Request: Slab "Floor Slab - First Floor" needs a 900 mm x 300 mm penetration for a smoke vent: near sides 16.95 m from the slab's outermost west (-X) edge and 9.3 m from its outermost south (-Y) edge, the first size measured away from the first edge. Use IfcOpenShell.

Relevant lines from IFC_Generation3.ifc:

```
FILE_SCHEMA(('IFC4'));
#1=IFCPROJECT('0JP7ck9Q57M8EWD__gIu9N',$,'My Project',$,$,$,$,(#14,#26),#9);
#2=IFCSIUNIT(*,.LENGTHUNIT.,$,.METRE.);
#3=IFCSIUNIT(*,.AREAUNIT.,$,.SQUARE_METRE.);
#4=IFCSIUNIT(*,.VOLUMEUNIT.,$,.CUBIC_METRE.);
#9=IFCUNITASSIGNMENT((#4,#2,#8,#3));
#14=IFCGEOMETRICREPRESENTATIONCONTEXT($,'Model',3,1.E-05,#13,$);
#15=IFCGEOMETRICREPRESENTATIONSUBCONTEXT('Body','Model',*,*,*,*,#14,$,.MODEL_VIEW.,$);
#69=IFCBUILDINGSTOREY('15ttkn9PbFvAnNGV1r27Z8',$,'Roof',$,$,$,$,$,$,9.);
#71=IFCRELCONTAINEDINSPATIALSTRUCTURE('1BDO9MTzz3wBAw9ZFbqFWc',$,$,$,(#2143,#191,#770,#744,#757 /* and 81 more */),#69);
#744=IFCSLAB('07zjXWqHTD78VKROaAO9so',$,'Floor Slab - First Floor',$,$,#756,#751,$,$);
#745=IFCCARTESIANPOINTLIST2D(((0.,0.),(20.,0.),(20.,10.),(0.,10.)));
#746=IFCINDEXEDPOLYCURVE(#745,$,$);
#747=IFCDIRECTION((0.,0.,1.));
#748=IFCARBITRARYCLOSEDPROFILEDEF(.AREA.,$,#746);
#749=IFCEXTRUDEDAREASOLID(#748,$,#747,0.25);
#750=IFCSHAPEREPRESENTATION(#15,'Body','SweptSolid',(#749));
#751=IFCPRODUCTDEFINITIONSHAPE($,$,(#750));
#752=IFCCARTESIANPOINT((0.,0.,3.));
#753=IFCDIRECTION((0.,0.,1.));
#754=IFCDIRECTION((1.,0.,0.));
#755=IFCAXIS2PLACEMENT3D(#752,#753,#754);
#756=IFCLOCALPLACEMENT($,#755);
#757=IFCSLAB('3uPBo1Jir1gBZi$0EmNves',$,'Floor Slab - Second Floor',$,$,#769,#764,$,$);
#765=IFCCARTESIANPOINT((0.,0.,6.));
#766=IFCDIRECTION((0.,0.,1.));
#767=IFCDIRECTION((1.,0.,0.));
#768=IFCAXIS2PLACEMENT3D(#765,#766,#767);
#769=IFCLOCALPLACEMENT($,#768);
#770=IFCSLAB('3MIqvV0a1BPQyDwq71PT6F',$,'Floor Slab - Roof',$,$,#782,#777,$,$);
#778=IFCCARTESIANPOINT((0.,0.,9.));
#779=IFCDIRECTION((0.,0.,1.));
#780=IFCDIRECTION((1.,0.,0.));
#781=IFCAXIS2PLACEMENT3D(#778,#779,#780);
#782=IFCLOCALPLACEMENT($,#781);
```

```python
import numpy as np
import ifcopenshell
import ifcopenshell.api.feature
import ifcopenshell.api.geometry
import ifcopenshell.api.root
import ifcopenshell.geom
import ifcopenshell.util.placement
import ifcopenshell.util.representation
import ifcopenshell.util.shape
import ifcopenshell.util.unit

model = ifcopenshell.open("IFC_Generation3.ifc")
unit_scale = ifcopenshell.util.unit.calculate_unit_scale(model)
settings = ifcopenshell.geom.settings()


def volume(element):
    """Net volume in cubic metres, openings subtracted."""
    shape = ifcopenshell.geom.create_shape(settings, element)
    return ifcopenshell.util.shape.get_volume(shape.geometry)


slab = model.by_guid("07zjXWqHTD78VKROaAO9so")
before = volume(slab)

# Extent in the slab's own axes, in metres. The edges named are its -X and -Y sides.
slab_shape = ifcopenshell.geom.create_shape(settings, slab)
vertices = ifcopenshell.util.shape.get_vertices(slab_shape.geometry)
x_min, y_min, bottom = vertices.min(axis=0)
top = vertices[:, 2].max()

opening = ifcopenshell.api.root.create_entity(model, ifc_class="IfcOpeningElement", name="Smoke vent opening", predefined_type="OPENING")
context = ifcopenshell.util.representation.get_context(model, "Model", "Body", "MODEL_VIEW")
width, depth = 0.9, 0.3
outline = [(0.0, 0.0), (width, 0.0), (width, depth), (0.0, depth), (0.0, 0.0)]
# Overshoot both faces by 50 mm so the cut is clean.
shape = ifcopenshell.api.geometry.add_slab_representation(
    model, context=context, depth=top - bottom + 0.1, polyline=outline
)
ifcopenshell.api.geometry.assign_representation(model, product=opening, representation=shape)

matrix = ifcopenshell.util.placement.get_local_placement(slab.ObjectPlacement)
matrix[:, 3] = matrix @ np.append(np.array([x_min + 16.95, y_min + 9.3, bottom - 0.05]) / unit_scale, 1.0)
ifcopenshell.api.geometry.edit_object_placement(model, product=opening, matrix=matrix, is_si=False)
ifcopenshell.api.feature.add_feature(model, feature=opening, element=slab)

after = volume(slab)

print(f"slab volume {before:.3f} -> {after:.3f} m3")

model.write("IFC_Generation3_v2.ifc")
```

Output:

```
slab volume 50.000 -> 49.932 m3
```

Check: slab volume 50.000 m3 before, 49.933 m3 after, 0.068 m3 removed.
